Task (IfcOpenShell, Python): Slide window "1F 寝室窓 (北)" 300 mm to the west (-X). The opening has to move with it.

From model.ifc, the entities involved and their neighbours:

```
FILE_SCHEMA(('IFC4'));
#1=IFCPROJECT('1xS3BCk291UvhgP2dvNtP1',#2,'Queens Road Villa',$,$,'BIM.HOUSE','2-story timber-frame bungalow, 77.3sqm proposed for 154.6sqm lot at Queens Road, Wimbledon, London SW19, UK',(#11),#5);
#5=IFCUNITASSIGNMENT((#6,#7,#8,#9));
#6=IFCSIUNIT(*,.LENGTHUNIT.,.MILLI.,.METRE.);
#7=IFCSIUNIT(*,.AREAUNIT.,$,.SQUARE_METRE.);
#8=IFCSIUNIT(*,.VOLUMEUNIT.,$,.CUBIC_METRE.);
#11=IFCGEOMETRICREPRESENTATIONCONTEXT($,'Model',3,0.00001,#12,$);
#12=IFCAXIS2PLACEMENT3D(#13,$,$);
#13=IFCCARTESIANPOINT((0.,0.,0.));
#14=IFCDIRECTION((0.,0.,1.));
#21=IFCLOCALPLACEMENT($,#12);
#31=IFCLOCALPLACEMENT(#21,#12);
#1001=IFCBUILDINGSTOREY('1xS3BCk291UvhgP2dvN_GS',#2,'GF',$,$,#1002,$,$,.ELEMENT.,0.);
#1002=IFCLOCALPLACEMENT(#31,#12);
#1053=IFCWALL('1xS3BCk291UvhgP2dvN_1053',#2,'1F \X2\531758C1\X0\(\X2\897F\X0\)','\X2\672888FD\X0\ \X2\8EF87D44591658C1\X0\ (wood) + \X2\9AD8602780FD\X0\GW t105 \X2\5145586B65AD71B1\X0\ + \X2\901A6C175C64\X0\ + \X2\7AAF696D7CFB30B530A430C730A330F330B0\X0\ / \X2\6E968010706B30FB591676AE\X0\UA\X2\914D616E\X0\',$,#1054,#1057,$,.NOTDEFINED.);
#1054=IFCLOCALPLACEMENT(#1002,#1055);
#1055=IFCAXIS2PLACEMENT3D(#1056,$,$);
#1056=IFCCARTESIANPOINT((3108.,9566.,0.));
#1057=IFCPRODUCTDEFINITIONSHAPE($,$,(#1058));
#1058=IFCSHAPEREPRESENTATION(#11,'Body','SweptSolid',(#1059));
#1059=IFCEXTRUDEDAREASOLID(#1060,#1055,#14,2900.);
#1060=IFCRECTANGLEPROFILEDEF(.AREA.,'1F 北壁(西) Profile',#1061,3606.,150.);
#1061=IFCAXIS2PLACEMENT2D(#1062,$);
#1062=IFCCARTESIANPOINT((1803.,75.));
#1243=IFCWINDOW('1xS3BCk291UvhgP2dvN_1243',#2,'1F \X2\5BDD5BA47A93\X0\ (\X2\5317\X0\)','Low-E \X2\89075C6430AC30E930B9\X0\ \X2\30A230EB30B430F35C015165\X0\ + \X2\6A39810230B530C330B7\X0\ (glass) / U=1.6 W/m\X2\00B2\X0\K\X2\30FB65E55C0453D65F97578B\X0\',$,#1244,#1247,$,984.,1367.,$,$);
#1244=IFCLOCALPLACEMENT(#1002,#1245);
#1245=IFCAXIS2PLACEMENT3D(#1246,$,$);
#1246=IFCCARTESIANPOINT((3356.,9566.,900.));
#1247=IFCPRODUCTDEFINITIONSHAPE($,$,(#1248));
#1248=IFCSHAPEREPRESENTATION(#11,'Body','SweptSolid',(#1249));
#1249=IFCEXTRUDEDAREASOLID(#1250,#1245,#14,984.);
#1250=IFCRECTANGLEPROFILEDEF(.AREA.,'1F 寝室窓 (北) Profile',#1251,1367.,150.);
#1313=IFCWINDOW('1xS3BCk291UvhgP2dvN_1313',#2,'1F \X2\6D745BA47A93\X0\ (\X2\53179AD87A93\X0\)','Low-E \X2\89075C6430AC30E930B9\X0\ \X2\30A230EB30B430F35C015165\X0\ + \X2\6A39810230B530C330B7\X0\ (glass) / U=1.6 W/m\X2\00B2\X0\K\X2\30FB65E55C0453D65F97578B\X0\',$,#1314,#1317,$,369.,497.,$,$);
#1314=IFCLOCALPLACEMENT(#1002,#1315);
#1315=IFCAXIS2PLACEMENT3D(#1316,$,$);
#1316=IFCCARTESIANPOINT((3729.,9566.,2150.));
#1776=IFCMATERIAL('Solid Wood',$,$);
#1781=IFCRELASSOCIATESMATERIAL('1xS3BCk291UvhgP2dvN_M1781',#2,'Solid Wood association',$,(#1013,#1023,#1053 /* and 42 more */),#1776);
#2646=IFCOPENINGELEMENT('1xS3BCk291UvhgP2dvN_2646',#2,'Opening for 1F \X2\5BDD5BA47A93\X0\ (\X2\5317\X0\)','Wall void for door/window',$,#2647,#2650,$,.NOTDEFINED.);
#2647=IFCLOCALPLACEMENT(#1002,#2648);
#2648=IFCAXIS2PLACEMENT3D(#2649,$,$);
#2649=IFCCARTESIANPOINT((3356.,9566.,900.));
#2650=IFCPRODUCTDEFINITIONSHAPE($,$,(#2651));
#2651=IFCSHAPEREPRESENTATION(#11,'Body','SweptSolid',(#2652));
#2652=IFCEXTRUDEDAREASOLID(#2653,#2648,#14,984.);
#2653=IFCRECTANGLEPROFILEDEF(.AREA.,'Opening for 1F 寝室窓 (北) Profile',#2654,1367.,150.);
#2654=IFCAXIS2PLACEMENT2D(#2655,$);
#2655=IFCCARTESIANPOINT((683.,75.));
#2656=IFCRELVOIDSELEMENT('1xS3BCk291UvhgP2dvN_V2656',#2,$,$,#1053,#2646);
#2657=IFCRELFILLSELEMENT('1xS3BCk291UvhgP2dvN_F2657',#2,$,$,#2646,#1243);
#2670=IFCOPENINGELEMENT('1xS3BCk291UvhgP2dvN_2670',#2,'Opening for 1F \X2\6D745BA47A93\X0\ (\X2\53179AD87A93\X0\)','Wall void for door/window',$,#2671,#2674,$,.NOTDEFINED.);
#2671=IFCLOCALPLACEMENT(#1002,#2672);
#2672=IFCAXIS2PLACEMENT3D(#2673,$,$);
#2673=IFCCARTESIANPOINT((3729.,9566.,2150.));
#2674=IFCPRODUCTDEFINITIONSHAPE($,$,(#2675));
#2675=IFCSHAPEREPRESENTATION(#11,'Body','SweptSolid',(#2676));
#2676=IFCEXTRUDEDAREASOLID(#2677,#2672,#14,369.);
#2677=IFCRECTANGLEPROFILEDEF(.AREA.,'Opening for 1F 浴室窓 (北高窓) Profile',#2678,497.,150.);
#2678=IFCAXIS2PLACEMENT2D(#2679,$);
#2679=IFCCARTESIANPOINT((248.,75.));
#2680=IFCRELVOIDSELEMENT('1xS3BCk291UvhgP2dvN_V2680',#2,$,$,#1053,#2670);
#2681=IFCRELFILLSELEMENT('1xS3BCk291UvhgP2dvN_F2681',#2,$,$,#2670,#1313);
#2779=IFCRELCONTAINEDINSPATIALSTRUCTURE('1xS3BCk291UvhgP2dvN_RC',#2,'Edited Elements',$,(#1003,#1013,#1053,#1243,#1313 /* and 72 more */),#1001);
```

```python
import ifcopenshell
import ifcopenshell.api.geometry
import ifcopenshell.util.placement
import ifcopenshell.util.unit

model = ifcopenshell.open("model.ifc")
unit_scale = ifcopenshell.util.unit.calculate_unit_scale(model)

window = model.by_id(1243)
opening = window.FillsVoids[0].RelatingOpeningElement
wall = opening.VoidsElements[0].RelatingBuildingElement

wall_matrix = ifcopenshell.util.placement.get_local_placement(wall.ObjectPlacement)
shift = wall_matrix[:3, 0] * -0.3 / unit_scale
before = ifcopenshell.util.placement.get_local_placement(window.ObjectPlacement)[:3, 3].copy()

# The window is not placed relative to its opening, so move both.
for product in (opening, window):
    matrix = ifcopenshell.util.placement.get_local_placement(product.ObjectPlacement)
    matrix[:3, 3] += shift
    ifcopenshell.api.geometry.edit_object_placement(model, product=product, matrix=matrix, is_si=False)

after = ifcopenshell.util.placement.get_local_placement(window.ObjectPlacement)[:3, 3]
print("window moved by", (after - before).round(3) + 0.0)

model.write("model-out.ifc")
```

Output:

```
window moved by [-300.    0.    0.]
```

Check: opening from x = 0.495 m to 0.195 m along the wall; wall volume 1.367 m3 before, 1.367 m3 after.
